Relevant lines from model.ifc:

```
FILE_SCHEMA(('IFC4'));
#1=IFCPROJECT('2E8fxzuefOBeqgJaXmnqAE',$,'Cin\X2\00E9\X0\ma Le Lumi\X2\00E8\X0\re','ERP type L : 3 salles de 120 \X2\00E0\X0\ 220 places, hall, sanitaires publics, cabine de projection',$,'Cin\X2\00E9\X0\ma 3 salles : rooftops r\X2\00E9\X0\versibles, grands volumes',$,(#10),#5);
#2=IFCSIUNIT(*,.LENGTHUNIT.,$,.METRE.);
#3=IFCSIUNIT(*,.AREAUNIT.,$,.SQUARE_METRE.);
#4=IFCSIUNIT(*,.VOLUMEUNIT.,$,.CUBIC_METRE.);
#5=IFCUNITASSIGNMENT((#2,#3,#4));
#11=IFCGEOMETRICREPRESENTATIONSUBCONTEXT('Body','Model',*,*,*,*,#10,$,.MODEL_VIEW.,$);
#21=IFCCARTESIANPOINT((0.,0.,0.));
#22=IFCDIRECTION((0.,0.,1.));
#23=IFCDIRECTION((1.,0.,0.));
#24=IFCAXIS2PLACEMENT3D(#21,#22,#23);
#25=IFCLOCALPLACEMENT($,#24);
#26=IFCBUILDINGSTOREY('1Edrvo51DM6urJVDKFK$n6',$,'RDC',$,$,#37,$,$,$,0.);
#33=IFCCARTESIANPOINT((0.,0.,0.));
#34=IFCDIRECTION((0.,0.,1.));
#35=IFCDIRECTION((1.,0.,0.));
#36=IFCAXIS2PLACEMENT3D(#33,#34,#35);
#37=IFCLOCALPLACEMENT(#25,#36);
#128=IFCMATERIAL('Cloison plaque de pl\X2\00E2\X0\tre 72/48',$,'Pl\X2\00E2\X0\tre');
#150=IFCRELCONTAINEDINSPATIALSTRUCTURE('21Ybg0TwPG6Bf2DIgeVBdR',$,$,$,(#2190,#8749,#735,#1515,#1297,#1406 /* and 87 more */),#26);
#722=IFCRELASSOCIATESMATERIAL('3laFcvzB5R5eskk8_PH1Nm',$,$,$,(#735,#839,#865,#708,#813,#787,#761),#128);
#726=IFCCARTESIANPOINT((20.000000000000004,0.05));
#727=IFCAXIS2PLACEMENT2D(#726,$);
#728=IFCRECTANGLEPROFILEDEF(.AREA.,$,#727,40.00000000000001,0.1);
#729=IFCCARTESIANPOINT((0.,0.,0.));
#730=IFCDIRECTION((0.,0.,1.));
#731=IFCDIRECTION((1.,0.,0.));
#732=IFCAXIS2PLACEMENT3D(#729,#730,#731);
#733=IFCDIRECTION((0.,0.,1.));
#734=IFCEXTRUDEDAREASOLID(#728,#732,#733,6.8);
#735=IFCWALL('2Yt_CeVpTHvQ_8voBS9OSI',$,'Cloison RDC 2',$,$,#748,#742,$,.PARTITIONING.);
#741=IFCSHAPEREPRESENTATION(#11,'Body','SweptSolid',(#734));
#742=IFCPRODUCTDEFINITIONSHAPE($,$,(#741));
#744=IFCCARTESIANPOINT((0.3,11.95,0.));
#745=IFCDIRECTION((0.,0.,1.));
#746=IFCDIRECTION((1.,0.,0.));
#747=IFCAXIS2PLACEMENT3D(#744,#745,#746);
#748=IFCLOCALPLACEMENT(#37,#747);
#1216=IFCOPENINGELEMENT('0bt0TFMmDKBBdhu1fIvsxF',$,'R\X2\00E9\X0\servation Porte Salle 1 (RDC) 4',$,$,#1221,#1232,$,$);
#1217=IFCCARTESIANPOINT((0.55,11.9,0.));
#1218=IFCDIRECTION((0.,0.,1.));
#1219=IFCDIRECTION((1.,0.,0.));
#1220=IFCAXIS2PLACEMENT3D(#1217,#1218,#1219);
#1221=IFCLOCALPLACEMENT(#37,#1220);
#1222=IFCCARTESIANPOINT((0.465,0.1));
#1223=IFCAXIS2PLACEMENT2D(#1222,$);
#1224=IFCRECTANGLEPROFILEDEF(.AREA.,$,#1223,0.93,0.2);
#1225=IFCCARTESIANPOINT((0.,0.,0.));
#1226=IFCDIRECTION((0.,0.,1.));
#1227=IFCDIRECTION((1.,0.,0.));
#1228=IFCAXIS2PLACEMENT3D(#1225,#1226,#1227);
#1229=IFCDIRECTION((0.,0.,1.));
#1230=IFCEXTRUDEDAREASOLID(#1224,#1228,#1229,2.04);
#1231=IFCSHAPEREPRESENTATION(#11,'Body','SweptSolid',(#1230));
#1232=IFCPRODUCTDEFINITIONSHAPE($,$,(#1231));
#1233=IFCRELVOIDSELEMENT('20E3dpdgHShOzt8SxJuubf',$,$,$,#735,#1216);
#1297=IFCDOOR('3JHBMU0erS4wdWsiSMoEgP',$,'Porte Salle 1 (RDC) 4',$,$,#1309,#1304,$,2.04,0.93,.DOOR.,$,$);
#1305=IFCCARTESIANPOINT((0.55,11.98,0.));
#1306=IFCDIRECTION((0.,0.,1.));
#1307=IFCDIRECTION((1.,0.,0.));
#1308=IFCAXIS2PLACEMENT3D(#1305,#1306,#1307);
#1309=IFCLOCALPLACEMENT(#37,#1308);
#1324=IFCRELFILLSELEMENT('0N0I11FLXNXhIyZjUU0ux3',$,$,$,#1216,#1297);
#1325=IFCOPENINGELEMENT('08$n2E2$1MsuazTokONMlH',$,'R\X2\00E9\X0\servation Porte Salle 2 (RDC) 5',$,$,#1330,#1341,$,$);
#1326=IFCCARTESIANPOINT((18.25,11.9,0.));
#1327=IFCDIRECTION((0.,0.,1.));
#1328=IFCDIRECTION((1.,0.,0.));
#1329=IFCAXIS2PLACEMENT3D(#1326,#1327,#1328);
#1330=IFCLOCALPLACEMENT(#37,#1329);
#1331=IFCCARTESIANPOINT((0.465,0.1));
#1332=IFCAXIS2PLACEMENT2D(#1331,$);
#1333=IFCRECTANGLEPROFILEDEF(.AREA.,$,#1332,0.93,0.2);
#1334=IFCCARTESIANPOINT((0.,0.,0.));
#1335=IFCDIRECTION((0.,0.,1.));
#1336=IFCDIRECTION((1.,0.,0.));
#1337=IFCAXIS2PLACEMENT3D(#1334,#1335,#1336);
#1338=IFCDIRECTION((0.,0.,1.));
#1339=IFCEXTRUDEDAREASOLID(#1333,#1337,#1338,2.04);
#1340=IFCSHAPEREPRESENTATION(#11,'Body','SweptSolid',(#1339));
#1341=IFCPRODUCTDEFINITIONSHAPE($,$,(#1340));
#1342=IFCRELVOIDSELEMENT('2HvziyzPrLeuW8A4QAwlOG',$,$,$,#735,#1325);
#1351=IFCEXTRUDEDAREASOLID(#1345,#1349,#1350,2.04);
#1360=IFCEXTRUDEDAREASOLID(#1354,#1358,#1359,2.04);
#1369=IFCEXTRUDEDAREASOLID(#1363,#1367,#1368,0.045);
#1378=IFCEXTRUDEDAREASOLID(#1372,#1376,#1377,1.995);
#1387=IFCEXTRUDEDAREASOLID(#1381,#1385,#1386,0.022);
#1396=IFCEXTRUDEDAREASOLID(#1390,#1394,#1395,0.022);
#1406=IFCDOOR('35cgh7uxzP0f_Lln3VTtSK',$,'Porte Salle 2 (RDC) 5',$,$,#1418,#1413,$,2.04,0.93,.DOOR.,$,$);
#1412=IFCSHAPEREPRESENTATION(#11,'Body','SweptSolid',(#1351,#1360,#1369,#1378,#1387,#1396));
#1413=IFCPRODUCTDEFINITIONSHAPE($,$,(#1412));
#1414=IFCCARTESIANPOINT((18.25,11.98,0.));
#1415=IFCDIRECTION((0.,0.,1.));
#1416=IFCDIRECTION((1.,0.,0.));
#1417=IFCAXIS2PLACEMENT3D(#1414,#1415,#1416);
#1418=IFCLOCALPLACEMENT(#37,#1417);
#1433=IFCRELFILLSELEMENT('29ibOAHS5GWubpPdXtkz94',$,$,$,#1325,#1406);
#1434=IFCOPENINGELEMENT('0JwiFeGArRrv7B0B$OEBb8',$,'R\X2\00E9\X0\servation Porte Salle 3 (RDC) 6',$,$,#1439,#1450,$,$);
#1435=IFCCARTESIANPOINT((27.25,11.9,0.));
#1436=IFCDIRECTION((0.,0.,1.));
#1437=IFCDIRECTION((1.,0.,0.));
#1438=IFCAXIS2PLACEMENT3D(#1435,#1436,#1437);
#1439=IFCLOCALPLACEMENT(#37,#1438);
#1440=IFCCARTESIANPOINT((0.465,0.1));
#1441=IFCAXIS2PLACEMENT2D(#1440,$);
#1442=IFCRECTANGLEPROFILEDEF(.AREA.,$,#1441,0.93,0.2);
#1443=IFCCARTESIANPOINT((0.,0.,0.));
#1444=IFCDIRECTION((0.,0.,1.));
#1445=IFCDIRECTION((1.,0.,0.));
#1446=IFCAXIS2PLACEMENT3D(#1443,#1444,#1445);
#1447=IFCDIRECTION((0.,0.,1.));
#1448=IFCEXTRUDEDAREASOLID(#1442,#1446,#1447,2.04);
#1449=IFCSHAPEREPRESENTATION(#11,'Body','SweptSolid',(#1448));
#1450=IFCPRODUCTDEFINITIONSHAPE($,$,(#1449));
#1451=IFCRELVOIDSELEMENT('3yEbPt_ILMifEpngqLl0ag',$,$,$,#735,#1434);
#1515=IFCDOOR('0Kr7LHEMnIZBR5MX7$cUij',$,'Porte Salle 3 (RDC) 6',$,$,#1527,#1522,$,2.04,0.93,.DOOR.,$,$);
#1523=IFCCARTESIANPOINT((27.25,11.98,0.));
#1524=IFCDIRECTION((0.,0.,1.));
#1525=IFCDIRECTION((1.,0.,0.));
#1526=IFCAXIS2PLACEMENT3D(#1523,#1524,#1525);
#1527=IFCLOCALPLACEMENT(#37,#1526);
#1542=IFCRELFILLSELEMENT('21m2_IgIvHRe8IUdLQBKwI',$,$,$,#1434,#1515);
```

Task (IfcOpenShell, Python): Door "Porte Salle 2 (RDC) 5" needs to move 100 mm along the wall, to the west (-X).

```python
import ifcopenshell
import ifcopenshell.api.geometry
import ifcopenshell.util.placement

model = ifcopenshell.open("model.ifc")

door = model.by_guid("35cgh7uxzP0f_Lln3VTtSK")
opening = door.FillsVoids[0].RelatingOpeningElement
wall = opening.VoidsElements[0].RelatingBuildingElement

wall_matrix = ifcopenshell.util.placement.get_local_placement(wall.ObjectPlacement)
shift = wall_matrix[:3, 0] * -0.1
before = ifcopenshell.util.placement.get_local_placement(door.ObjectPlacement)[:3, 3].copy()

# The door is not placed relative to its opening, so move both.
for product in (opening, door):
    matrix = ifcopenshell.util.placement.get_local_placement(product.ObjectPlacement)
    matrix[:3, 3] += shift
    ifcopenshell.api.geometry.edit_object_placement(model, product=product, matrix=matrix, is_si=False)

after = ifcopenshell.util.placement.get_local_placement(door.ObjectPlacement)[:3, 3]
print("door moved by", (after - before).round(3) + 0.0)

model.write("model_edited.ifc")
```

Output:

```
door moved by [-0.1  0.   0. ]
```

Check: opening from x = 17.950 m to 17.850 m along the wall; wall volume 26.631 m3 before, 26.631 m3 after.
